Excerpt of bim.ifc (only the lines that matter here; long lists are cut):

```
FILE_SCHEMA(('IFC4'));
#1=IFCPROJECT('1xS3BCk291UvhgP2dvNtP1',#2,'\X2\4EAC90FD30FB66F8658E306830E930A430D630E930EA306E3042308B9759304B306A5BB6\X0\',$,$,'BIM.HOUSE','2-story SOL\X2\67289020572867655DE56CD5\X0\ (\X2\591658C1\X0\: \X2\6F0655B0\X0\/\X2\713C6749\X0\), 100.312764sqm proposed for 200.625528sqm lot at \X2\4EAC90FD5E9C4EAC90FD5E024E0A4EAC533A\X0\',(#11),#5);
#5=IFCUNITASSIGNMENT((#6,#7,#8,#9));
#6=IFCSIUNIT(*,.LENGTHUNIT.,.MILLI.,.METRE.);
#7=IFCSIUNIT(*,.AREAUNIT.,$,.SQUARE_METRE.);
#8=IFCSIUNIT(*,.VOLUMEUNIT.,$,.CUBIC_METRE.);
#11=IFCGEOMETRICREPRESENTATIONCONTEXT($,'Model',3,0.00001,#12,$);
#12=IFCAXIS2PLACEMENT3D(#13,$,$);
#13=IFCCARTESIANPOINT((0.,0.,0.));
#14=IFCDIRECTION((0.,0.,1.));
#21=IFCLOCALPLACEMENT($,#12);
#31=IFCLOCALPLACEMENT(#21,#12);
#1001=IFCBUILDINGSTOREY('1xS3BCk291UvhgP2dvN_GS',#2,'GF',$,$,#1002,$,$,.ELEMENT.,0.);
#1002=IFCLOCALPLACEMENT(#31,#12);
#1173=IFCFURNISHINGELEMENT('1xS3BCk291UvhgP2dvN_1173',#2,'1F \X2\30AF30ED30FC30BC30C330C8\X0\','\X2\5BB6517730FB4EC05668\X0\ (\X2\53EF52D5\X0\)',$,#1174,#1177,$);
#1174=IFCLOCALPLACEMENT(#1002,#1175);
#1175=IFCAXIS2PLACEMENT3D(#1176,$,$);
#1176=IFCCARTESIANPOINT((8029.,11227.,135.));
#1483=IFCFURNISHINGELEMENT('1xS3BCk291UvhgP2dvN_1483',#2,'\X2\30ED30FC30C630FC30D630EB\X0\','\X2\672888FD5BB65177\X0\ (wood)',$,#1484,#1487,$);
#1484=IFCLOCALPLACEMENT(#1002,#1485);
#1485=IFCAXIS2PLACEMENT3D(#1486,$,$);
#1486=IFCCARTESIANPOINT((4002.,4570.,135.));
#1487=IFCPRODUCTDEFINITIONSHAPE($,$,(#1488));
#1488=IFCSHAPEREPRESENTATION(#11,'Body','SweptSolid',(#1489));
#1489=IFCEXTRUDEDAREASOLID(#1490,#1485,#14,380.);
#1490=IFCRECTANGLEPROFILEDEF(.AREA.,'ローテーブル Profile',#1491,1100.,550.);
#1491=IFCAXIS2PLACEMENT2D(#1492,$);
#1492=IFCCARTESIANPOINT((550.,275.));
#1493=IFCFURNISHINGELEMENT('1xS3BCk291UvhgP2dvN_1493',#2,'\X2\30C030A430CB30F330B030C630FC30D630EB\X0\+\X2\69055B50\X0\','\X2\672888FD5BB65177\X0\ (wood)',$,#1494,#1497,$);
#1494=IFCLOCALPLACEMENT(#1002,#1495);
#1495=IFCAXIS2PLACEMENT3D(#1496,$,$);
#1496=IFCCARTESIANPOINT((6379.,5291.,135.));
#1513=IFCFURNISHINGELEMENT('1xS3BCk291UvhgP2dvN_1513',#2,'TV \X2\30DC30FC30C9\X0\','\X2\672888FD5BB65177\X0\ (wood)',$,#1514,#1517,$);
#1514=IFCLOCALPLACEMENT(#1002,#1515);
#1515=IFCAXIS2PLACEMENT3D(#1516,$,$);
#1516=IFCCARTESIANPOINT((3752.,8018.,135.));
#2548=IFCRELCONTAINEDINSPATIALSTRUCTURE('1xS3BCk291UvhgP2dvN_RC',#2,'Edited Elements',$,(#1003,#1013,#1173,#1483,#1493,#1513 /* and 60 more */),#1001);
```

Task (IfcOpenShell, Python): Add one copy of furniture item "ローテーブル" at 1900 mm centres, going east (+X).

```python
import numpy as np
import ifcopenshell
import ifcopenshell.api.geometry
import ifcopenshell.api.root
import ifcopenshell.util.element
import ifcopenshell.util.placement

model = ifcopenshell.open("bim.ifc")


def reuse_history(source, copy):
    """copy_class also copies each property set's owner history, people and application; keep the originals."""
    for rel in copy.IsDefinedBy:
        if rel.is_a("IfcRelDefinesByProperties") and (history := rel.RelatingPropertyDefinition.OwnerHistory):
            rel.RelatingPropertyDefinition.OwnerHistory = source.OwnerHistory
            ifcopenshell.util.element.remove_deep2(model, history)


source = model.by_guid("1xS3BCk291UvhgP2dvN_1483")
base = ifcopenshell.util.placement.get_local_placement(source.ObjectPlacement)
step = np.array([1.0, 0.0, 0.0]) * 1900.0

for i in range(1, 2):
    copy = ifcopenshell.api.root.copy_class(model, product=source)
    copy.Representation = ifcopenshell.util.element.copy_deep(
        model, source.Representation, exclude=["IfcGeometricRepresentationContext", "IfcRepresentationMap"]
    )
    reuse_history(source, copy)
    matrix = base.copy()
    matrix[:3, 3] += i * step
    print("added at", matrix[:3, 3].round(3) + 0.0)
    ifcopenshell.api.geometry.edit_object_placement(model, product=copy, matrix=matrix, is_si=False)

model.write("bim-out.ifc")
```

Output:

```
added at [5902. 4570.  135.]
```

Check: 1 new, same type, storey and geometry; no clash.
